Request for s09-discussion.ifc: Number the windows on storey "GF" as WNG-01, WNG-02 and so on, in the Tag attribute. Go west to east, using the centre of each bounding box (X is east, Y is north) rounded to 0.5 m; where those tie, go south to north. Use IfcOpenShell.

First a look at what the model holds.

```python
import ifcopenshell
import ifcopenshell.util.element
import ifcopenshell.util.placement

model = ifcopenshell.open("s09-discussion.ifc")
print(model.schema)
storey = next(s for s in model.by_type("IfcBuildingStorey") if s.Name == "GF")
windows = [e for e in ifcopenshell.util.element.get_decomposition(storey) if e.is_a("IfcWindow")]
for e in sorted(windows, key=lambda e: e.id()):
    origin = ifcopenshell.util.placement.get_local_placement(e.ObjectPlacement)[:3, 3]
    print(e.id(), e.Tag, e.Name, origin.round(2) + 0.0, sep=" | ")
```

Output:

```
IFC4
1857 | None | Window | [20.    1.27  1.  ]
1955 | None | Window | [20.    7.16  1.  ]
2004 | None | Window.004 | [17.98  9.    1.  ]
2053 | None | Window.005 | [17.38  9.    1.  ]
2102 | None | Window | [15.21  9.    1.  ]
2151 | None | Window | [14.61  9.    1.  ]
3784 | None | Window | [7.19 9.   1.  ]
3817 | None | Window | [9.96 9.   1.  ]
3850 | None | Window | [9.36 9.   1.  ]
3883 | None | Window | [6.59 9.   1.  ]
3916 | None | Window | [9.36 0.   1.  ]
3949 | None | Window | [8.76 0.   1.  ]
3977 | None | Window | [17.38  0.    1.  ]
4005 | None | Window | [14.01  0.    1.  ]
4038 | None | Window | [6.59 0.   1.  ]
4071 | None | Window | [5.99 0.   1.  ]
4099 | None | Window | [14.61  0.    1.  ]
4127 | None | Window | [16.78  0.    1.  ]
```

```python
import ifcopenshell
import ifcopenshell.geom
import ifcopenshell.util.element
import ifcopenshell.util.shape

model = ifcopenshell.open("s09-discussion.ifc")
settings = ifcopenshell.geom.settings()
settings.set("use-world-coords", True)


def centre(element):
    shape = ifcopenshell.geom.create_shape(settings, element)
    return ifcopenshell.util.shape.get_bbox_centroid(shape.geometry)


storey = next(s for s in model.by_type("IfcBuildingStorey") if s.Name == "GF")
windows = [e for e in ifcopenshell.util.element.get_decomposition(storey) if e.is_a("IfcWindow")]

# Insertion points can sit at a corner or the storey origin, so sort by the geometry (in metres).
centres = {e: centre(e) for e in windows}
windows.sort(key=lambda e: (round(centres[e][0] / 0.5), centres[e][1]))

for i, e in enumerate(windows, start=1):
    number = f"WNG-{i:02d}"
    e.Tag = number
    print(e.id(), number)

model.write("s09-discussion_updated.ifc")
```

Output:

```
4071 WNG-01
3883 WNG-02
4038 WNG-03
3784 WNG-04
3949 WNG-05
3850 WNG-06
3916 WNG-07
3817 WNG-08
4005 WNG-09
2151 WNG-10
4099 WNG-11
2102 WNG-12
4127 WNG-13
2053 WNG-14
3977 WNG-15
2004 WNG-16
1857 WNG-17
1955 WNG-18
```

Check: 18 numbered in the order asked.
